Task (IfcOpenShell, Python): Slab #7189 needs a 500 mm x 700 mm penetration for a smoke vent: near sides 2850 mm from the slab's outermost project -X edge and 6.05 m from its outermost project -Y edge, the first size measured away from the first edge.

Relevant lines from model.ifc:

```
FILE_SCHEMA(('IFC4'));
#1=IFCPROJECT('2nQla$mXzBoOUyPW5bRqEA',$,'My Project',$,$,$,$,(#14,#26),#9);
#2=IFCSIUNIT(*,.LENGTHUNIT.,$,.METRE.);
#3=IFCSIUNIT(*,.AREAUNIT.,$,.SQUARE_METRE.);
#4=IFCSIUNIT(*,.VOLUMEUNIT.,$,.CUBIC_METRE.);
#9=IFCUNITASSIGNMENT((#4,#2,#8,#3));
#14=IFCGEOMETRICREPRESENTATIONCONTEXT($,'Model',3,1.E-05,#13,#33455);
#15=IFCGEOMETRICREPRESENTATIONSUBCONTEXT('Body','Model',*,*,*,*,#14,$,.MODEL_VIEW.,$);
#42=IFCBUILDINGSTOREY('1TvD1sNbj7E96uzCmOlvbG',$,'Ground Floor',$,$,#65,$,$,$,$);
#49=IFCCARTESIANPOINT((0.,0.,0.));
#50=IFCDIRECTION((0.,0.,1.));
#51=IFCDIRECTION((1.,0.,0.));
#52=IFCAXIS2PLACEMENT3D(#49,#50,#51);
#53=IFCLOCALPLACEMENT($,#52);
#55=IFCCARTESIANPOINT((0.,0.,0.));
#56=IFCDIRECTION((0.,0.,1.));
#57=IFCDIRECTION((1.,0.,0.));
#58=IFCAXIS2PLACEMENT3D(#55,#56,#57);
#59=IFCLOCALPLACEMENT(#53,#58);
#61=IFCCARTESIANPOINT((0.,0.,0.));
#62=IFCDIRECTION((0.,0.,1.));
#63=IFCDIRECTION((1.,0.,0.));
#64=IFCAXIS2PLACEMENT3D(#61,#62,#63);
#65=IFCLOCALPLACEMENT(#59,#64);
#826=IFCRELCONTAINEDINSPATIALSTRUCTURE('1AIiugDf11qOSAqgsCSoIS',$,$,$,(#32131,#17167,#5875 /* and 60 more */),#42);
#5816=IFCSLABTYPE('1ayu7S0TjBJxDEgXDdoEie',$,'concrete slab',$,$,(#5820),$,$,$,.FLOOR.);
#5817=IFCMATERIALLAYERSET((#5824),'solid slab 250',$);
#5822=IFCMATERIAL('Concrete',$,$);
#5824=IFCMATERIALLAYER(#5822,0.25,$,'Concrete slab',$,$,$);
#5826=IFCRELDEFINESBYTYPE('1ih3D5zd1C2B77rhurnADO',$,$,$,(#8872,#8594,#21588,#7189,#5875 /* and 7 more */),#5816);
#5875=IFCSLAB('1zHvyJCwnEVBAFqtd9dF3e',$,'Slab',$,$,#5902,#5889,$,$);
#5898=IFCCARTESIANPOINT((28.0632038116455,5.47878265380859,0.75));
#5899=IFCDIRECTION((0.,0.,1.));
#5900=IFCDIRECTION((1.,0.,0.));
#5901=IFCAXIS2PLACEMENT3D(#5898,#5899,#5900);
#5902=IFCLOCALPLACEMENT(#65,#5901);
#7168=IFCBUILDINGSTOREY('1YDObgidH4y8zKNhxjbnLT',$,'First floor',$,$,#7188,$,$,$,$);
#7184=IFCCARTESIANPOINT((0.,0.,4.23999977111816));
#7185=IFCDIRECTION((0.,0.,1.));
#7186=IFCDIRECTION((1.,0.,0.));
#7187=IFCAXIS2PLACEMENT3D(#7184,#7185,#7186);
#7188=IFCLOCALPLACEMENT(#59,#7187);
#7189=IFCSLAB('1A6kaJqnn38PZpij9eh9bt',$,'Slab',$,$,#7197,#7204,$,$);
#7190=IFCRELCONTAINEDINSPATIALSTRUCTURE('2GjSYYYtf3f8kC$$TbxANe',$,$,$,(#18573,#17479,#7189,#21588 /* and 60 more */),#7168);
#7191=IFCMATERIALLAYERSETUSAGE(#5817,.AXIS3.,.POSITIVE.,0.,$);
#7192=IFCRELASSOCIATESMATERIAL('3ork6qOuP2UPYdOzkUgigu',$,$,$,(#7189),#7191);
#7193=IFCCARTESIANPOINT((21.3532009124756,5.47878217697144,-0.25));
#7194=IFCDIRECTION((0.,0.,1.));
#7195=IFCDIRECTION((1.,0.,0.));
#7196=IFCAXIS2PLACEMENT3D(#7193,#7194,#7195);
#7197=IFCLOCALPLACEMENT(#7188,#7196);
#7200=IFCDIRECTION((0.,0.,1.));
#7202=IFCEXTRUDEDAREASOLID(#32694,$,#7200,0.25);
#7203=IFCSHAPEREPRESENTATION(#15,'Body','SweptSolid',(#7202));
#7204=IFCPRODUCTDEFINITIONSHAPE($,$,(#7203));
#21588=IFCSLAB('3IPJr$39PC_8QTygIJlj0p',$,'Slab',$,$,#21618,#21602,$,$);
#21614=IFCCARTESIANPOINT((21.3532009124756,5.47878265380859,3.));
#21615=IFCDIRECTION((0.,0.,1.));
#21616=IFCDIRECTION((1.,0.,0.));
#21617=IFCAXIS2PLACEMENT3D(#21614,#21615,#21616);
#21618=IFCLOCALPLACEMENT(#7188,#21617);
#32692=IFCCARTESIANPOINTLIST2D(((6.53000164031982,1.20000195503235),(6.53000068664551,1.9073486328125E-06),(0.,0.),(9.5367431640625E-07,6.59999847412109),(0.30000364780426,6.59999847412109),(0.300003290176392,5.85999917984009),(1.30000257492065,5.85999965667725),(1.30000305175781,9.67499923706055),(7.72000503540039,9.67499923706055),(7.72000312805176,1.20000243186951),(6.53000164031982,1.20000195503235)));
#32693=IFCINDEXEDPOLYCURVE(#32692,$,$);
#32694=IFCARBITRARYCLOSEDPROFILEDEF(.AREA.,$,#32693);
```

```python
import numpy as np
import ifcopenshell
import ifcopenshell.api.feature
import ifcopenshell.api.geometry
import ifcopenshell.api.root
import ifcopenshell.geom
import ifcopenshell.util.placement
import ifcopenshell.util.representation
import ifcopenshell.util.shape
import ifcopenshell.util.unit

model = ifcopenshell.open("model.ifc")
unit_scale = ifcopenshell.util.unit.calculate_unit_scale(model)
settings = ifcopenshell.geom.settings()


def volume(element):
    """Net volume in cubic metres, openings subtracted."""
    shape = ifcopenshell.geom.create_shape(settings, element)
    return ifcopenshell.util.shape.get_volume(shape.geometry)


slab = model.by_guid("1A6kaJqnn38PZpij9eh9bt")
before = volume(slab)

# Extent in the slab's own axes, in metres. The edges named are its -X and -Y sides.
slab_shape = ifcopenshell.geom.create_shape(settings, slab)
vertices = ifcopenshell.util.shape.get_vertices(slab_shape.geometry)
x_min, y_min, bottom = vertices.min(axis=0)
top = vertices[:, 2].max()

opening = ifcopenshell.api.root.create_entity(model, ifc_class="IfcOpeningElement", name="Smoke vent opening", predefined_type="OPENING")
context = ifcopenshell.util.representation.get_context(model, "Model", "Body", "MODEL_VIEW")
width, depth = 0.5, 0.7
outline = [(0.0, 0.0), (width, 0.0), (width, depth), (0.0, depth), (0.0, 0.0)]
# Overshoot both faces by 50 mm so the cut is clean.
shape = ifcopenshell.api.geometry.add_slab_representation(
    model, context=context, depth=top - bottom + 0.1, polyline=outline
)
ifcopenshell.api.geometry.assign_representation(model, product=opening, representation=shape)

matrix = ifcopenshell.util.placement.get_local_placement(slab.ObjectPlacement)
matrix[:, 3] = matrix @ np.append(np.array([x_min + 2.85, y_min + 6.05, bottom - 0.05]) / unit_scale, 1.0)
ifcopenshell.api.geometry.edit_object_placement(model, product=opening, matrix=matrix, is_si=False)
ifcopenshell.api.feature.add_feature(model, feature=opening, element=slab)

after = volume(slab)

print(f"slab volume {before:.3f} -> {after:.3f} m3")

model.write("model_updated.ifc")
```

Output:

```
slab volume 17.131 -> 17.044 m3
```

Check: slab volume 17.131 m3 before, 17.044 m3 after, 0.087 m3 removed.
